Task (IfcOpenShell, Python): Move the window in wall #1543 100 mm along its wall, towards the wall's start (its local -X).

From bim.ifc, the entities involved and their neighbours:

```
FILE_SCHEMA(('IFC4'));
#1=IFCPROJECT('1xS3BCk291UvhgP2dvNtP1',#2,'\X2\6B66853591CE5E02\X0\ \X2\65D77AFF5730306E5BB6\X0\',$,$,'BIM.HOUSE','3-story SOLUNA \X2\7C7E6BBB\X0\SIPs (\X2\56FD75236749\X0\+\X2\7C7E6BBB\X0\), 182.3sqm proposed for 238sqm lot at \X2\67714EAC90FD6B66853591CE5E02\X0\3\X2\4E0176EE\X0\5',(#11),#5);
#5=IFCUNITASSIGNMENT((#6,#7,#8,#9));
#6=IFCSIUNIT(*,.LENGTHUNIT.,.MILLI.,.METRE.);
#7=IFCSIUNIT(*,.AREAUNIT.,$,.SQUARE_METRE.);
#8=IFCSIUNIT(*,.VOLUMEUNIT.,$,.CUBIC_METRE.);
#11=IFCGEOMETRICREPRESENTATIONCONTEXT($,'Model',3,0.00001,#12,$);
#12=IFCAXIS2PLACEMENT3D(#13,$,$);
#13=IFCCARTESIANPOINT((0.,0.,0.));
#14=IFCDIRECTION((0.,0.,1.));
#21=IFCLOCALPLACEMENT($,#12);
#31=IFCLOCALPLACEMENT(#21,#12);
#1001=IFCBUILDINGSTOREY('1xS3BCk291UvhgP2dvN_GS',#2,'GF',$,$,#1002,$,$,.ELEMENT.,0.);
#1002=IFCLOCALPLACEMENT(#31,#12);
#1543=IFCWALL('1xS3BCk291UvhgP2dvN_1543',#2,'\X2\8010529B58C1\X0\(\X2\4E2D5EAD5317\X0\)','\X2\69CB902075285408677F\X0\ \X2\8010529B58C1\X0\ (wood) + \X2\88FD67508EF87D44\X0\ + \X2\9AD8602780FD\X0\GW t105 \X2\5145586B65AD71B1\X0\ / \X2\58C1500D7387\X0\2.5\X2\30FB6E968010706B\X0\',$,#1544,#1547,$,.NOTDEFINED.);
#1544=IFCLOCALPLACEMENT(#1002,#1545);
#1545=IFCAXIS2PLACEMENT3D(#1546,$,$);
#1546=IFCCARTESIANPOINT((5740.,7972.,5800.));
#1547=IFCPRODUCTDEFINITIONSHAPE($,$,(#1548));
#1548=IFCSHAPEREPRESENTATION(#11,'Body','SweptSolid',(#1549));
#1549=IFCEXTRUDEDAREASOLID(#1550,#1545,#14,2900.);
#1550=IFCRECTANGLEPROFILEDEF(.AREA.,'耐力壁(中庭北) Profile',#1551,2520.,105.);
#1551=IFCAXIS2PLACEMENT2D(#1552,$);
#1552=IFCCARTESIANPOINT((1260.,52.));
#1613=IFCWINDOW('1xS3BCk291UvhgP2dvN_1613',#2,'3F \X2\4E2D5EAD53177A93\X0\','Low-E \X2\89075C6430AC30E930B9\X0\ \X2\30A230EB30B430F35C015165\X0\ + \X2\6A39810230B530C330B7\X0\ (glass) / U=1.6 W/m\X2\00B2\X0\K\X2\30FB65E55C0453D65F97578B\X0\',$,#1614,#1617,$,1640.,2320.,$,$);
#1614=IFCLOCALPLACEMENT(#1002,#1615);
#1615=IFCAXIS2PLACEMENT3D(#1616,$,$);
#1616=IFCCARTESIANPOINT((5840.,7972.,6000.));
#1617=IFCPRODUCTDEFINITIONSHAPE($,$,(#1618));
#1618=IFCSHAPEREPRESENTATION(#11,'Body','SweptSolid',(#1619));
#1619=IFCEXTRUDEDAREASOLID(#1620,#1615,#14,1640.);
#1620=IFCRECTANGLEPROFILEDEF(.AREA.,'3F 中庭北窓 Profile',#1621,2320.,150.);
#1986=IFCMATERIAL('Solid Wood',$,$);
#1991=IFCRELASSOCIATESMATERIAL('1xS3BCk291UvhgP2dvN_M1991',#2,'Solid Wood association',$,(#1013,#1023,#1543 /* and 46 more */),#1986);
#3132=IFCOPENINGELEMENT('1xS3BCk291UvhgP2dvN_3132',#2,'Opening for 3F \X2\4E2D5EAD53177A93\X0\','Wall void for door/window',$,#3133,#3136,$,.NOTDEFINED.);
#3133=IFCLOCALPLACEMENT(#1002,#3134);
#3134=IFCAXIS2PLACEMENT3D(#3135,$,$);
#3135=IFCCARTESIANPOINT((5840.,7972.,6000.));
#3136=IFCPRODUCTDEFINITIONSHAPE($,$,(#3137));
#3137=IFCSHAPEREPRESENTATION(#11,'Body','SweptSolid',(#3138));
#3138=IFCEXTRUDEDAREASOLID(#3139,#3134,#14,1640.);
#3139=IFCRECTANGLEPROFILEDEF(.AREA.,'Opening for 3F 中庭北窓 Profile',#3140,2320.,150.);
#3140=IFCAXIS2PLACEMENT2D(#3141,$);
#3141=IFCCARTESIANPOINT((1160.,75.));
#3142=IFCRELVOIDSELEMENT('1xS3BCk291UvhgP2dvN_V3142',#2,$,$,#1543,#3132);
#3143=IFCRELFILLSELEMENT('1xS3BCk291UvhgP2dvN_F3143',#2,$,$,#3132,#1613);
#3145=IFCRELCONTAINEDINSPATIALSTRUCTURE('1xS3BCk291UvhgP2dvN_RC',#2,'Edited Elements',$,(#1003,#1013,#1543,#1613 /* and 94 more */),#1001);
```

```python
import ifcopenshell
import ifcopenshell.api.geometry
import ifcopenshell.util.placement
import ifcopenshell.util.unit

model = ifcopenshell.open("bim.ifc")
unit_scale = ifcopenshell.util.unit.calculate_unit_scale(model)

window = model.by_guid("1xS3BCk291UvhgP2dvN_1613")
opening = window.FillsVoids[0].RelatingOpeningElement
wall = opening.VoidsElements[0].RelatingBuildingElement

wall_matrix = ifcopenshell.util.placement.get_local_placement(wall.ObjectPlacement)
shift = wall_matrix[:3, 0] * -0.1 / unit_scale
before = ifcopenshell.util.placement.get_local_placement(window.ObjectPlacement)[:3, 3].copy()

# The window is not placed relative to its opening, so move both.
for product in (opening, window):
    matrix = ifcopenshell.util.placement.get_local_placement(product.ObjectPlacement)
    matrix[:3, 3] += shift
    ifcopenshell.api.geometry.edit_object_placement(model, product=product, matrix=matrix, is_si=False)

after = ifcopenshell.util.placement.get_local_placement(window.ObjectPlacement)[:3, 3]
print("window moved by", (after - before).round(3) + 0.0)

model.write("bim_rev.ifc")
```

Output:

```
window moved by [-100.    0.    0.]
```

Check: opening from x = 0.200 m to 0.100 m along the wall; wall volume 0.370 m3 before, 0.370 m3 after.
